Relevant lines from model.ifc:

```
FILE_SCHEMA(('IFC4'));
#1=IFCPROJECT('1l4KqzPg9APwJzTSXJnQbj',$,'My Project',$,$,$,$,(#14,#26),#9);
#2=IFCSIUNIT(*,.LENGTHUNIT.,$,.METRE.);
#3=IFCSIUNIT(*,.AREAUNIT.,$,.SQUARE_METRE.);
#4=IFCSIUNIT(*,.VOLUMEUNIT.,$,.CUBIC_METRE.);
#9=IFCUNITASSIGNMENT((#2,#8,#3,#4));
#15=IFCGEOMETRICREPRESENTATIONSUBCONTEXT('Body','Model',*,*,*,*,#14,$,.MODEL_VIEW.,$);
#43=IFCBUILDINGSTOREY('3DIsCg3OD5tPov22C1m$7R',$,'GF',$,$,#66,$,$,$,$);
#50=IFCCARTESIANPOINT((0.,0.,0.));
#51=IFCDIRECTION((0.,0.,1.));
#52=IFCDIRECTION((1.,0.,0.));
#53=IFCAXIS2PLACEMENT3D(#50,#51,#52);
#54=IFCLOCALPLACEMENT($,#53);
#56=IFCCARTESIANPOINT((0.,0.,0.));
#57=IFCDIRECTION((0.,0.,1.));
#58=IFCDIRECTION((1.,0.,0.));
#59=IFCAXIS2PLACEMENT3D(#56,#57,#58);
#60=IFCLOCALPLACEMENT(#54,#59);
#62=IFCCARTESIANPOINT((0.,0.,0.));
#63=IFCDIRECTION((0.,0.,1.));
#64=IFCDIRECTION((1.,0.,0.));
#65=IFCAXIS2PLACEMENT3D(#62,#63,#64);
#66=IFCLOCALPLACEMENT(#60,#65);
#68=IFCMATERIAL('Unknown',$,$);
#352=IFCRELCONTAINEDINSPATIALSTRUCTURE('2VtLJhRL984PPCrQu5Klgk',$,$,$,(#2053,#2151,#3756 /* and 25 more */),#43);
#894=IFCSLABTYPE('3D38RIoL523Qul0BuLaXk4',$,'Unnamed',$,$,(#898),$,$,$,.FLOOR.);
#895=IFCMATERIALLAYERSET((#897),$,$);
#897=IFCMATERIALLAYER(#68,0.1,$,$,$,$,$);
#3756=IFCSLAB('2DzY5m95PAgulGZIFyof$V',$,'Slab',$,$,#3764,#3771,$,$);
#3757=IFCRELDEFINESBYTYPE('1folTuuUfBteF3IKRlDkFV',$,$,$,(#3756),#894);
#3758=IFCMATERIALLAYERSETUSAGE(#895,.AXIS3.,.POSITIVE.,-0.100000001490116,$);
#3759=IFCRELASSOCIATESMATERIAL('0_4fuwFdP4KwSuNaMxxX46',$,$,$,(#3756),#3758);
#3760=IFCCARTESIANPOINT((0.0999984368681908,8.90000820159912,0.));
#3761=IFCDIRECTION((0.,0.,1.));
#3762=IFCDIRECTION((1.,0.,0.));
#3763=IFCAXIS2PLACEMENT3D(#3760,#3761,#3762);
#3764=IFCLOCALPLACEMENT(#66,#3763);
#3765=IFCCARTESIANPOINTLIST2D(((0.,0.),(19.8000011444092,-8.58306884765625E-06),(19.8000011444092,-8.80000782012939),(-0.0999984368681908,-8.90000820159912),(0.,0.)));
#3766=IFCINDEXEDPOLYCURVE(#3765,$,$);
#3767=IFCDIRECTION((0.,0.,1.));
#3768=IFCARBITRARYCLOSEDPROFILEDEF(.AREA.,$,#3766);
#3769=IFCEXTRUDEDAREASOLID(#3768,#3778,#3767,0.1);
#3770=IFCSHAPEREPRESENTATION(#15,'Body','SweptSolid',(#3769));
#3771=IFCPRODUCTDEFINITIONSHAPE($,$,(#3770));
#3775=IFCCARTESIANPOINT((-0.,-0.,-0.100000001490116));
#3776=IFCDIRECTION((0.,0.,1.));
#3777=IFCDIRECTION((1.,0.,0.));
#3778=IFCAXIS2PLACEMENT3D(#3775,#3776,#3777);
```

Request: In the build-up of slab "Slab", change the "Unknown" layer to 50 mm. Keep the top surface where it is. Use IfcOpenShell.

```python
import ifcopenshell
import ifcopenshell.util.element
import ifcopenshell.util.representation
import ifcopenshell.util.unit

model = ifcopenshell.open("model.ifc")
unit_scale = ifcopenshell.util.unit.calculate_unit_scale(model)

layer_set = model.by_id(895)
layer = next(l for l in layer_set.MaterialLayers if l.Material and l.Material.Name == "Unknown")
change = 0.05 / unit_scale - layer.LayerThickness
layer.LayerThickness += change

# Geometry does not follow the layer set by itself.
slabs = [e for e in ifcopenshell.util.element.get_elements_by_material(model, layer_set) if e.is_a("IfcSlab")]
for slab in sorted(slabs, key=lambda e: e.id()):
    body = ifcopenshell.util.representation.get_representation(slab, "Model", "Body")
    solid = body.Items[0]
    old_depth = solid.Depth
    solid.Depth += change
    # Extruded upwards: lower the start of the extrusion so the top stays.
    x, y, z = solid.Position.Location.Coordinates
    solid.Position.Location = model.createIfcCartesianPoint((x, y, z - change))
    print(slab.id(), f"{old_depth:g} -> {solid.Depth:g}")

# The layers are counted up from the underside, which has moved.
for usage in {ifcopenshell.util.element.get_material(slab) for slab in slabs}:
    usage.OffsetFromReferenceLine -= change

model.write("model_rev.ifc")
```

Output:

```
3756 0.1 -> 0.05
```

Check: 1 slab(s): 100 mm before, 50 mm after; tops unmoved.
